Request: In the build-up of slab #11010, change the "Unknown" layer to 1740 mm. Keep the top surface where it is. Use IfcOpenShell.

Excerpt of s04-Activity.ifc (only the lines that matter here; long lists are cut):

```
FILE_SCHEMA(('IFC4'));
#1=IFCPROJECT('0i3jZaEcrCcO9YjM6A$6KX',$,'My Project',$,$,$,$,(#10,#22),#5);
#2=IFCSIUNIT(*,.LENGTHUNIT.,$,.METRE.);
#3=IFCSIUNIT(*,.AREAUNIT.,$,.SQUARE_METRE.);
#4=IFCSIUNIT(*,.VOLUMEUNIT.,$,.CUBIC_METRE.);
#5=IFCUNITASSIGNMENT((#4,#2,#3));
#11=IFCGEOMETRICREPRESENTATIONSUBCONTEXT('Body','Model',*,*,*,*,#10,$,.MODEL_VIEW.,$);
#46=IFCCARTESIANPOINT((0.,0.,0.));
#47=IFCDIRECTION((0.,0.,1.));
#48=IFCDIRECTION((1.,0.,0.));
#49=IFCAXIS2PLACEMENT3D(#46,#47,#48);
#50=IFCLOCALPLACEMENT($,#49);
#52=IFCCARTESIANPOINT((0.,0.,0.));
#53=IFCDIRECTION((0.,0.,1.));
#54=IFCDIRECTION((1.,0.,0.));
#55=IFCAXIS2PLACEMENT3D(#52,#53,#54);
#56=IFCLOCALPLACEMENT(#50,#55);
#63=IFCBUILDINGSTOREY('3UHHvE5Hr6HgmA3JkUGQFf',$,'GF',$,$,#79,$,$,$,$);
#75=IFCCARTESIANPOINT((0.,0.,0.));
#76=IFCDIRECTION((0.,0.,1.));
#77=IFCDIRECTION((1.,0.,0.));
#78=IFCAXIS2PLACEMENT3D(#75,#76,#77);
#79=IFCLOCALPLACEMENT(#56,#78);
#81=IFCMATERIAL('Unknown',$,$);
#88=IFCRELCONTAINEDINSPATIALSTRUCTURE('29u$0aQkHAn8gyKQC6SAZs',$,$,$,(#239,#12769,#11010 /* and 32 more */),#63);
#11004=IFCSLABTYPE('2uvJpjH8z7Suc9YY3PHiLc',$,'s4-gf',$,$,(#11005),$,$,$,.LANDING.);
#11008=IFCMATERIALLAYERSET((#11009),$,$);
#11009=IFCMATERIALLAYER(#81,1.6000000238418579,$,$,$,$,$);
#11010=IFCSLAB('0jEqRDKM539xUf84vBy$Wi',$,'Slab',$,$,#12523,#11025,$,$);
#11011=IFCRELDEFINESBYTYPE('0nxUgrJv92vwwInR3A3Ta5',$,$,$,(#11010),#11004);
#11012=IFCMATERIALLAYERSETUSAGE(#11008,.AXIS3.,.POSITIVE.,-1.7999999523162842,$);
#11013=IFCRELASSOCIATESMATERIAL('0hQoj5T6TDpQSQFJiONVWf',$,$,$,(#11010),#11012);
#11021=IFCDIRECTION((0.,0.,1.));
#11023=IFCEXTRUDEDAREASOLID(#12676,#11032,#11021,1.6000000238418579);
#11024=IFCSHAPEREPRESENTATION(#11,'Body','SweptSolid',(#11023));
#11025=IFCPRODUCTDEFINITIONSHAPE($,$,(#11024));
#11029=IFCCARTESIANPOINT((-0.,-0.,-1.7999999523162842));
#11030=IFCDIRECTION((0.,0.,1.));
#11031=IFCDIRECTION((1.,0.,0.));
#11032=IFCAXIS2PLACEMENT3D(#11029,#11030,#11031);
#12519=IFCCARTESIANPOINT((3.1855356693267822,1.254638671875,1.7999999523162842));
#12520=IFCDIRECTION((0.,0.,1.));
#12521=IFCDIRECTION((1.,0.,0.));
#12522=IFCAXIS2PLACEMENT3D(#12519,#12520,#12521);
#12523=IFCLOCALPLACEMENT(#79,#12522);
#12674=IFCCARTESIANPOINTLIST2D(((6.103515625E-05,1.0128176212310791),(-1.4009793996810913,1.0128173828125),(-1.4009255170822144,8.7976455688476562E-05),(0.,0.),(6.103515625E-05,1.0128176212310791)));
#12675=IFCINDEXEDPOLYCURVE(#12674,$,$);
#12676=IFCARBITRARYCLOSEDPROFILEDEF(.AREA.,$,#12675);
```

```python
import ifcopenshell
import ifcopenshell.util.element
import ifcopenshell.util.representation

model = ifcopenshell.open("s04-Activity.ifc")

layer_set = model.by_id(11008)
layer = next(l for l in layer_set.MaterialLayers if l.Material and l.Material.Name == "Unknown")
change = 1.74 - layer.LayerThickness
layer.LayerThickness += change

# Geometry does not follow the layer set by itself.
slabs = [e for e in ifcopenshell.util.element.get_elements_by_material(model, layer_set) if e.is_a("IfcSlab")]
for slab in sorted(slabs, key=lambda e: e.id()):
    body = ifcopenshell.util.representation.get_representation(slab, "Model", "Body")
    solid = body.Items[0]
    old_depth = solid.Depth
    solid.Depth += change
    # Extruded upwards: lower the start of the extrusion so the top stays.
    x, y, z = solid.Position.Location.Coordinates
    solid.Position.Location = model.createIfcCartesianPoint((x, y, z - change))
    print(slab.id(), f"{old_depth:g} -> {solid.Depth:g}")

# The layers are counted up from the underside, which has moved.
for usage in {ifcopenshell.util.element.get_material(slab) for slab in slabs}:
    usage.OffsetFromReferenceLine -= change

model.write("s04-Activity_rev.ifc")
```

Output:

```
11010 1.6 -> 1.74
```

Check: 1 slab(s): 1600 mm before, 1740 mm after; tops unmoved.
